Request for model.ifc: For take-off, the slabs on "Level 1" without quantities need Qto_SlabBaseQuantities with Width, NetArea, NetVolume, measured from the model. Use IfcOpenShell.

First a look at what the model holds.

```python
import ifcopenshell
import ifcopenshell.util.element
import ifcopenshell.util.unit

model = ifcopenshell.open("model.ifc")
print(model.schema)
for unit_type in ("LENGTHUNIT", "AREAUNIT", "VOLUMEUNIT"):
    print(unit_type, ifcopenshell.util.unit.calculate_unit_scale(model, unit_type))
storey = next(s for s in model.by_type("IfcBuildingStorey") if s.Name == "Level 1")
slabs = [e for e in ifcopenshell.util.element.get_decomposition(storey) if e.is_a("IfcSlab")]
for e in sorted(slabs, key=lambda e: e.id()):
    print(e.id(), e.is_a(), e.Name, list(ifcopenshell.util.element.get_psets(e, qtos_only=True)), sep=" | ")
```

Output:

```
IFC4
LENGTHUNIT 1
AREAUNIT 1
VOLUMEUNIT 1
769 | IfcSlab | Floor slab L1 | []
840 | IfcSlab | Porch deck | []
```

```python
import ifcopenshell
import ifcopenshell.api.pset
import ifcopenshell.geom
import ifcopenshell.util.element
import ifcopenshell.util.shape
import ifcopenshell.util.unit

model = ifcopenshell.open("model.ifc")
unit_scale = ifcopenshell.util.unit.calculate_unit_scale(model)
area_scale = ifcopenshell.util.unit.calculate_unit_scale(model, "AREAUNIT")
volume_scale = ifcopenshell.util.unit.calculate_unit_scale(model, "VOLUMEUNIT")
settings = ifcopenshell.geom.settings()

storey = next(s for s in model.by_type("IfcBuildingStorey") if s.Name == "Level 1")
slabs = [e for e in ifcopenshell.util.element.get_decomposition(storey) if e.is_a("IfcSlab")]

for e in sorted(slabs, key=lambda e: e.id()):
    if ifcopenshell.util.element.get_psets(e, qtos_only=True, should_inherit=False):
        continue
    # Geometry comes back in metres, in the element's own axes.
    shape = ifcopenshell.geom.create_shape(settings, e)
    values = {
        "Width": ifcopenshell.util.shape.get_z(shape.geometry) / unit_scale,
        "NetArea": ifcopenshell.util.shape.get_footprint_area(shape.geometry) / area_scale,
        "NetVolume": ifcopenshell.util.shape.get_volume(shape.geometry) / volume_scale,
    }
    qto = ifcopenshell.api.pset.add_qto(model, product=e, name="Qto_SlabBaseQuantities")
    ifcopenshell.api.pset.edit_qto(model, qto=qto, properties=values)
    print(e.id(), {k: round(v, 3) for k, v in values.items()})

model.write("model_rev.ifc")
```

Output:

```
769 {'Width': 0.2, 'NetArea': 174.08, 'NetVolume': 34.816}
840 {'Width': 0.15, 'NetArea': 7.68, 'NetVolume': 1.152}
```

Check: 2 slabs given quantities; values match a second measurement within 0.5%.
